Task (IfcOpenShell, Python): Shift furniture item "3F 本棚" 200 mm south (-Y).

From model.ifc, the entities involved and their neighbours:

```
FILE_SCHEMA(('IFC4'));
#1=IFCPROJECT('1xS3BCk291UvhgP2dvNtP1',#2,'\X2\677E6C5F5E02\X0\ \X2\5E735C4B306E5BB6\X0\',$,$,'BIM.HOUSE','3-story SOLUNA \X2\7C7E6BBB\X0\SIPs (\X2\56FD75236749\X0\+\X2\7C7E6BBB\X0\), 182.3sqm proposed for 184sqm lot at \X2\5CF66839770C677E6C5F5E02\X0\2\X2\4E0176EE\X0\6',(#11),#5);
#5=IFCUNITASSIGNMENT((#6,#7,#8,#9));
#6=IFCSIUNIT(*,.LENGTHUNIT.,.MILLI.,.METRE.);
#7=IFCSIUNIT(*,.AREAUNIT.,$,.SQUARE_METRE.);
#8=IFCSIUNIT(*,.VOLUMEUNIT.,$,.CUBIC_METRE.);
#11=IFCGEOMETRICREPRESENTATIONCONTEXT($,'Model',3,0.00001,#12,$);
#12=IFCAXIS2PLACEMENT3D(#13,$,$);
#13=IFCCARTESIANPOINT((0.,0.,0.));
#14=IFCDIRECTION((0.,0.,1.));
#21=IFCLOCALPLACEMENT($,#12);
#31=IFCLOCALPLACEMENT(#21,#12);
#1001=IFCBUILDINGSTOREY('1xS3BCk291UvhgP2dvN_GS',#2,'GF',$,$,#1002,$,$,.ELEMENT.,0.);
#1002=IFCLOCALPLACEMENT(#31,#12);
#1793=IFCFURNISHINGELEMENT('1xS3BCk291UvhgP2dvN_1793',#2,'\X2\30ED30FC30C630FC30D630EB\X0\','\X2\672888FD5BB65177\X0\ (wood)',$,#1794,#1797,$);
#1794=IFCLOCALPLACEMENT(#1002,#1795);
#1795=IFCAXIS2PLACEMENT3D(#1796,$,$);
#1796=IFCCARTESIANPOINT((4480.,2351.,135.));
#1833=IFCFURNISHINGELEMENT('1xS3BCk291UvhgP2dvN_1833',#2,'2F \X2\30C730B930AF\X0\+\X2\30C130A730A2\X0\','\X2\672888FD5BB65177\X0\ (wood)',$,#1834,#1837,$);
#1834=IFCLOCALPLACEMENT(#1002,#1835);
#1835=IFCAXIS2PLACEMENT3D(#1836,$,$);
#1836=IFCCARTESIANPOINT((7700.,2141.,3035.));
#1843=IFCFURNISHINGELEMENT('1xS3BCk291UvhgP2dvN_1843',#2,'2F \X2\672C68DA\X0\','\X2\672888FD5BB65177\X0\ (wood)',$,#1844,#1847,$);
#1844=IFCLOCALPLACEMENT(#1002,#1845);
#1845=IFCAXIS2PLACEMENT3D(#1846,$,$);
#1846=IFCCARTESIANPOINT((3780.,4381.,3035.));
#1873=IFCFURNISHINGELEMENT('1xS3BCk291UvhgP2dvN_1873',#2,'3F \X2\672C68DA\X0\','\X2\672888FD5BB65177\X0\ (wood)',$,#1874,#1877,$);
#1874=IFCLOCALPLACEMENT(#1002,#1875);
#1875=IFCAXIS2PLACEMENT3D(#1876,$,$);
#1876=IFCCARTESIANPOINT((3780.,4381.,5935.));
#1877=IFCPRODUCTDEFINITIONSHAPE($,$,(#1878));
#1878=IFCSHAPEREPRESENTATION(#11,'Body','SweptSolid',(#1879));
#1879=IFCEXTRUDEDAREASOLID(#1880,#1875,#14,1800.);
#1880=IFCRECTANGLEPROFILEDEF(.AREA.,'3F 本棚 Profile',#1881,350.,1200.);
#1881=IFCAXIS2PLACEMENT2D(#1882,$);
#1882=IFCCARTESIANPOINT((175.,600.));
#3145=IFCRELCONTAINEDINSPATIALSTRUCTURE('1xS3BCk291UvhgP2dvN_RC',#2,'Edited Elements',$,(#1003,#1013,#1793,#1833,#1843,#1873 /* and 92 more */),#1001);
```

```python
import ifcopenshell
import ifcopenshell.api.geometry
import ifcopenshell.util.placement
import ifcopenshell.util.unit

model = ifcopenshell.open("model.ifc")
unit_scale = ifcopenshell.util.unit.calculate_unit_scale(model)

item = model.by_guid("1xS3BCk291UvhgP2dvN_1873")
matrix = ifcopenshell.util.placement.get_local_placement(item.ObjectPlacement)
matrix[1, 3] -= 0.2 / unit_scale
ifcopenshell.api.geometry.edit_object_placement(model, product=item, matrix=matrix, is_si=False)

print(ifcopenshell.util.placement.get_local_placement(item.ObjectPlacement).round(3) + 0.0)

model.write("model_edited.ifc")
```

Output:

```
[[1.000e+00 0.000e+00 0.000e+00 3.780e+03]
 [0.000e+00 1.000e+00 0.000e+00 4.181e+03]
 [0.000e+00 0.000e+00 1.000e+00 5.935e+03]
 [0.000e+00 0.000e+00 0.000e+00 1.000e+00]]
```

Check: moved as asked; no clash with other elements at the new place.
